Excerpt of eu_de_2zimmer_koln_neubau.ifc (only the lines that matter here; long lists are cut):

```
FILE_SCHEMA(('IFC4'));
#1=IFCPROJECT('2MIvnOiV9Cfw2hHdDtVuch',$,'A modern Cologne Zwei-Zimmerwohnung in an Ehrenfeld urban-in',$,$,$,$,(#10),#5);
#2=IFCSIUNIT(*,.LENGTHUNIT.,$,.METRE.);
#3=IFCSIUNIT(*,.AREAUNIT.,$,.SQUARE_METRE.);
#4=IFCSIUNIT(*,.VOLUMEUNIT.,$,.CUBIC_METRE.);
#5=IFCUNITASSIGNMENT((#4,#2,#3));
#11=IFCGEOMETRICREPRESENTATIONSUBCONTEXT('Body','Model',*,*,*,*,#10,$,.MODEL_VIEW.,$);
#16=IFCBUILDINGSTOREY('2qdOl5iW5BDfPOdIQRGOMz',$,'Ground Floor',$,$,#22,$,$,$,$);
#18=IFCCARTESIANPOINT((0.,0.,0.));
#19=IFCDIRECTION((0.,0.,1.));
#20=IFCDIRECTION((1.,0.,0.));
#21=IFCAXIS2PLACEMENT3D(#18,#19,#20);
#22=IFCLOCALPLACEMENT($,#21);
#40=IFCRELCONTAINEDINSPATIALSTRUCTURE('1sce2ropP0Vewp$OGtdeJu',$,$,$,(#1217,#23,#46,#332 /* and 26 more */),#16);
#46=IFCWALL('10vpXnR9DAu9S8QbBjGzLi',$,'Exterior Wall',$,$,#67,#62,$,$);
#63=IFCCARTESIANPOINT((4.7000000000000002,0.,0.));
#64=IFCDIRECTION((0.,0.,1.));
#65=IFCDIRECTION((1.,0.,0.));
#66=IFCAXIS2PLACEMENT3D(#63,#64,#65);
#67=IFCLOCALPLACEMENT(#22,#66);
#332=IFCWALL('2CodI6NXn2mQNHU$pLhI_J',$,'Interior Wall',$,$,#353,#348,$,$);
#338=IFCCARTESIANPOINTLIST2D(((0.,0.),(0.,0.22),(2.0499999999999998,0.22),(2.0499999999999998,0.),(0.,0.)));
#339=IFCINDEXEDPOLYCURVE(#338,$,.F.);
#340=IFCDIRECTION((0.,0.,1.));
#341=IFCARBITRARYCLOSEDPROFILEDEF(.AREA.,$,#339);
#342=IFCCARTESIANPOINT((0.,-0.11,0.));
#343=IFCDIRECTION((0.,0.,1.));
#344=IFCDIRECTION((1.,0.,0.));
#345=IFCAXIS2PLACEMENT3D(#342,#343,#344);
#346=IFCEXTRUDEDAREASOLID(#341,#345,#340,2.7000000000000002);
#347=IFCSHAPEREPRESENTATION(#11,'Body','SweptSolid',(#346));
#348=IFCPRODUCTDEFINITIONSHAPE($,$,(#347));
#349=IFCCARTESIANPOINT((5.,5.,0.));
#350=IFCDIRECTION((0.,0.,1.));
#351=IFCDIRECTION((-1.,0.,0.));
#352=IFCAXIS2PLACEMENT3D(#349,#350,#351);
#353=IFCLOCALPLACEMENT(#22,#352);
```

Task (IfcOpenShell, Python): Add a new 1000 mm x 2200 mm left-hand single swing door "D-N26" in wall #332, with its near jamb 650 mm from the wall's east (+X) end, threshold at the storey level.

```python
import numpy as np
import ifcopenshell
import ifcopenshell.api.feature
import ifcopenshell.api.geometry
import ifcopenshell.api.root
import ifcopenshell.api.spatial
import ifcopenshell.geom
import ifcopenshell.util.element
import ifcopenshell.util.placement
import ifcopenshell.util.representation
import ifcopenshell.util.shape
import ifcopenshell.util.unit

model = ifcopenshell.open("eu_de_2zimmer_koln_neubau.ifc")
unit_scale = ifcopenshell.util.unit.calculate_unit_scale(model)
settings = ifcopenshell.geom.settings()


def volume(element):
    """Net volume in cubic metres, openings subtracted."""
    shape = ifcopenshell.geom.create_shape(settings, element)
    return ifcopenshell.util.shape.get_volume(shape.geometry)


wall = model.by_guid("2CodI6NXn2mQNHU$pLhI_J")
storey = ifcopenshell.util.element.get_container(wall, ifc_class="IfcBuildingStorey")
context = ifcopenshell.util.representation.get_context(model, "Model", "Body", "MODEL_VIEW")
before = volume(wall)

width, height, from_end, sill = 1, 2.2, 0.65, 0.0  # metres

# The wall runs along its own X axis, and the end named is its -X end.
wall_shape = ifcopenshell.geom.create_shape(settings, wall)
x, y, z = ifcopenshell.util.shape.get_vertices(wall_shape.geometry).T
start = x.min() + from_end
face, thickness = float(y.min()), float(y.max() - y.min())
wall_matrix = ifcopenshell.util.placement.get_local_placement(wall.ObjectPlacement)
level = ifcopenshell.util.placement.get_local_placement(storey.ObjectPlacement)[2, 3]


def in_wall(x, y):
    """Placement at x, y metres in the wall's axes, at sill height."""
    matrix = wall_matrix.copy()
    matrix[:, 3] = wall_matrix @ np.array([x / unit_scale, y / unit_scale, 0.0, 1.0])
    matrix[2, 3] = level + sill / unit_scale
    return matrix


# Opening: a box that overshoots both wall faces by 50 mm.
opening = ifcopenshell.api.root.create_entity(model, ifc_class="IfcOpeningElement", predefined_type="OPENING")
box = ifcopenshell.api.geometry.add_wall_representation(
    model, context=context, length=width, height=height, thickness=thickness + 0.1
)
ifcopenshell.api.geometry.assign_representation(model, product=opening, representation=box)
ifcopenshell.api.geometry.edit_object_placement(model, product=opening, matrix=in_wall(start, face - 0.05), is_si=False)
ifcopenshell.api.feature.add_feature(model, feature=opening, element=wall)

door = ifcopenshell.api.root.create_entity(model, ifc_class="IfcDoor", name="D-N26", predefined_type="DOOR")
door.OverallWidth, door.OverallHeight = width / unit_scale, height / unit_scale
door.OperationType = "SINGLE_SWING_LEFT"
body = ifcopenshell.api.geometry.add_door_representation(
    model,
    context=context,
    overall_width=door.OverallWidth,
    overall_height=door.OverallHeight,
    operation_type="SINGLE_SWING_LEFT",
    lining_properties={"LiningDepth": thickness / unit_scale, "ThresholdDepth": thickness / unit_scale},
)
ifcopenshell.api.geometry.assign_representation(model, product=door, representation=body)
ifcopenshell.api.spatial.assign_container(model, products=[door], relating_structure=storey)
ifcopenshell.api.feature.add_filling(model, opening=opening, element=door)

# The lining spans the wall, so the door starts at the wall face.
ifcopenshell.api.geometry.edit_object_placement(model, product=door, matrix=in_wall(start, face), is_si=False)

after = volume(wall)

print(f"wall volume {before:.3f} -> {after:.3f} m3")

model.write("eu_de_2zimmer_koln_neubau_edited.ifc")
```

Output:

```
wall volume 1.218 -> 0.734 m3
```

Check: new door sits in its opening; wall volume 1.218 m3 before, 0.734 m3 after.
